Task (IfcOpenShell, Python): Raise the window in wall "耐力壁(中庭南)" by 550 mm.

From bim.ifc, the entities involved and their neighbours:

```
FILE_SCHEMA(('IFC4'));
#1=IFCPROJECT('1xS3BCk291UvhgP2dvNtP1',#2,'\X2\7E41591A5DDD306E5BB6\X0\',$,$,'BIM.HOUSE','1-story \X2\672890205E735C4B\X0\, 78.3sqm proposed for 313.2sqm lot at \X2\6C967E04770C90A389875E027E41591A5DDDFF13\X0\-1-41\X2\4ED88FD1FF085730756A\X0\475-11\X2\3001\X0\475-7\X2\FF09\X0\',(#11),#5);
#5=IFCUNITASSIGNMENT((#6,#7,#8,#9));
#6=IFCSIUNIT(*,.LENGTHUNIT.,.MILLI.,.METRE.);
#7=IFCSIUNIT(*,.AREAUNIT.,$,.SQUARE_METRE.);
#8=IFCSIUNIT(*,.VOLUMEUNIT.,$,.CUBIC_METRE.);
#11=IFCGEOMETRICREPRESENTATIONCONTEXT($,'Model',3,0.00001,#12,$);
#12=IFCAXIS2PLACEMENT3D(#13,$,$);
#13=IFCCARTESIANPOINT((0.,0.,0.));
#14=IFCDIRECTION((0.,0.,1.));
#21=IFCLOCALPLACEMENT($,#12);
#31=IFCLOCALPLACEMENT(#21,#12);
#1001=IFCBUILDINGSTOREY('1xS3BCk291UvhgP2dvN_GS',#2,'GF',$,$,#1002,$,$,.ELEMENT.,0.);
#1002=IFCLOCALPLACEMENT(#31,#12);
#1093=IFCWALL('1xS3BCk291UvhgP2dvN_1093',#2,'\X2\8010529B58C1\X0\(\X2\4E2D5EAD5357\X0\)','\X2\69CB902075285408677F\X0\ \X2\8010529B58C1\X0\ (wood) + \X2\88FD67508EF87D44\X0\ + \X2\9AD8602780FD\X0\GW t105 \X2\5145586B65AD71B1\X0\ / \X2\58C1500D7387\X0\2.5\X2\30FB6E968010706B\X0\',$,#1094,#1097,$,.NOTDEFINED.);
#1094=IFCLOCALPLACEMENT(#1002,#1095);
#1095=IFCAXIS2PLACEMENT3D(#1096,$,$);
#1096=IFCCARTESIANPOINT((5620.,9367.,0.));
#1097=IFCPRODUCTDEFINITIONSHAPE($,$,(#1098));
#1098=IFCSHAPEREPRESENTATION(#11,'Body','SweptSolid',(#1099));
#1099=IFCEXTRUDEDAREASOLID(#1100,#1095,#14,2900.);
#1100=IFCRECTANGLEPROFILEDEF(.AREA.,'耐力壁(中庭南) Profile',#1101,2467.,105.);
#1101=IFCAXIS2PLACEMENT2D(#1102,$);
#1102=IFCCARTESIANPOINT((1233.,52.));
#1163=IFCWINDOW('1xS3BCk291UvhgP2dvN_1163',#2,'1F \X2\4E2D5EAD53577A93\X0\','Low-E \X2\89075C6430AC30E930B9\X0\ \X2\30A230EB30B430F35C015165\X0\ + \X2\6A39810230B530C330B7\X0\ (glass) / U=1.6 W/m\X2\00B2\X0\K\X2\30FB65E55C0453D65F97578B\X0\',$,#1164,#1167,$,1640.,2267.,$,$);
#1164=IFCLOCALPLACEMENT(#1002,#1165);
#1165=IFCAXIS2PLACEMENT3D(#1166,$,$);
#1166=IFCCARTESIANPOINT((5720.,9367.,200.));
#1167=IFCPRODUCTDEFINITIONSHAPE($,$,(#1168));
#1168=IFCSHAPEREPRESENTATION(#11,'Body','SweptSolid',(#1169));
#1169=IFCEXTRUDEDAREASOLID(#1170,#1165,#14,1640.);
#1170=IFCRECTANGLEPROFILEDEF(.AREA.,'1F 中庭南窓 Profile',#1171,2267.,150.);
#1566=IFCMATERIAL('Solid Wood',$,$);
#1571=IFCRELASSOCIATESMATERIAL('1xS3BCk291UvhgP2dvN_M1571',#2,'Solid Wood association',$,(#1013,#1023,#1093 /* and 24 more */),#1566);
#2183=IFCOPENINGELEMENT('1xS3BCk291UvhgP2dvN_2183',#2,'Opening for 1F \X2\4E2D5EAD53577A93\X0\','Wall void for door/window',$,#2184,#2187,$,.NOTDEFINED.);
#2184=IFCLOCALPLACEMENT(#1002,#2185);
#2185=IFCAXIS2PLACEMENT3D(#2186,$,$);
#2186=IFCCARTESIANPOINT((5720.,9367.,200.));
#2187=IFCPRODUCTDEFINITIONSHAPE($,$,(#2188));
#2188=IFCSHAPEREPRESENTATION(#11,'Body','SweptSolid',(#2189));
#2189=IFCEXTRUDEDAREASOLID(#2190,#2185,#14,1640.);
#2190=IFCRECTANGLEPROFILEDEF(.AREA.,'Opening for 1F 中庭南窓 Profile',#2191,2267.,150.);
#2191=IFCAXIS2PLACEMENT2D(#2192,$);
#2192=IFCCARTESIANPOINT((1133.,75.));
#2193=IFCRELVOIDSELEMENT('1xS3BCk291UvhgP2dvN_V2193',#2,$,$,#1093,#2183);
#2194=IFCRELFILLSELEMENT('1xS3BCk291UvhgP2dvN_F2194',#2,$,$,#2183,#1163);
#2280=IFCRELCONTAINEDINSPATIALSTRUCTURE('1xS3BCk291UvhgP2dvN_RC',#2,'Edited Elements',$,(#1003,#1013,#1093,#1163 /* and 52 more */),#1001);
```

```python
import numpy as np
import ifcopenshell
import ifcopenshell.api.geometry
import ifcopenshell.util.placement
import ifcopenshell.util.unit

model = ifcopenshell.open("bim.ifc")
unit_scale = ifcopenshell.util.unit.calculate_unit_scale(model)

window = model.by_guid("1xS3BCk291UvhgP2dvN_1163")
opening = window.FillsVoids[0].RelatingOpeningElement
dz = 550.0

shift = np.array([0.0, 0.0, dz])
# The window is not placed relative to its opening, so move both.
for product in (opening, window):
    matrix = ifcopenshell.util.placement.get_local_placement(product.ObjectPlacement)
    matrix[:3, 3] += shift
    ifcopenshell.api.geometry.edit_object_placement(model, product=product, matrix=matrix, is_si=False)

print(f"moved by {dz * unit_scale:+.3f} m")

model.write("bim-out.ifc")
```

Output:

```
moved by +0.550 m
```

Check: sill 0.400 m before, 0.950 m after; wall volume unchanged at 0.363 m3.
